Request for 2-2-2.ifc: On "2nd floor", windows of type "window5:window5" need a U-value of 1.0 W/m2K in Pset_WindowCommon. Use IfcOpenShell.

First a look at what the model holds.

```python
import ifcopenshell
import ifcopenshell.util.element

model = ifcopenshell.open("2-2-2.ifc")
print(model.schema)
storey = next(s for s in model.by_type("IfcBuildingStorey") if s.Name == "2nd floor")
windows = [e for e in ifcopenshell.util.element.get_decomposition(storey) if e.is_a("IfcWindow")]
seen = {}
for e in windows:
    element_type = ifcopenshell.util.element.get_type(e)
    key = (element_type.Name if element_type != e and element_type else None, ifcopenshell.util.element.get_pset(e, "Pset_WindowCommon", "ThermalTransmittance"))
    seen[key] = seen.get(key, 0) + 1
for (name, value), count in sorted(seen.items(), key=str):
    print(count, "x", name, "|", value)
```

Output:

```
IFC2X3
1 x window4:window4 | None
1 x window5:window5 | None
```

```python
import ifcopenshell
import ifcopenshell.api.pset
import ifcopenshell.util.element

model = ifcopenshell.open("2-2-2.ifc")

storey = next(s for s in model.by_type("IfcBuildingStorey") if s.Name == "2nd floor")
windows = [e for e in ifcopenshell.util.element.get_decomposition(storey) if e.is_a("IfcWindow")]

count = 0
for e in windows:
    element_type = ifcopenshell.util.element.get_type(e)
    if element_type in (None, e) or element_type.Name != "window5:window5":
        continue
    # add_pset returns the element's existing set when there is one.
    pset = ifcopenshell.api.pset.add_pset(model, product=e, name="Pset_WindowCommon")
    ifcopenshell.api.pset.edit_pset(model, pset=pset, properties={"ThermalTransmittance": 1.0})
    count += 1

print(count, "windows updated")

model.write("2-2-2_updated.ifc")
```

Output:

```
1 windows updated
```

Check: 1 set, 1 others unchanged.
